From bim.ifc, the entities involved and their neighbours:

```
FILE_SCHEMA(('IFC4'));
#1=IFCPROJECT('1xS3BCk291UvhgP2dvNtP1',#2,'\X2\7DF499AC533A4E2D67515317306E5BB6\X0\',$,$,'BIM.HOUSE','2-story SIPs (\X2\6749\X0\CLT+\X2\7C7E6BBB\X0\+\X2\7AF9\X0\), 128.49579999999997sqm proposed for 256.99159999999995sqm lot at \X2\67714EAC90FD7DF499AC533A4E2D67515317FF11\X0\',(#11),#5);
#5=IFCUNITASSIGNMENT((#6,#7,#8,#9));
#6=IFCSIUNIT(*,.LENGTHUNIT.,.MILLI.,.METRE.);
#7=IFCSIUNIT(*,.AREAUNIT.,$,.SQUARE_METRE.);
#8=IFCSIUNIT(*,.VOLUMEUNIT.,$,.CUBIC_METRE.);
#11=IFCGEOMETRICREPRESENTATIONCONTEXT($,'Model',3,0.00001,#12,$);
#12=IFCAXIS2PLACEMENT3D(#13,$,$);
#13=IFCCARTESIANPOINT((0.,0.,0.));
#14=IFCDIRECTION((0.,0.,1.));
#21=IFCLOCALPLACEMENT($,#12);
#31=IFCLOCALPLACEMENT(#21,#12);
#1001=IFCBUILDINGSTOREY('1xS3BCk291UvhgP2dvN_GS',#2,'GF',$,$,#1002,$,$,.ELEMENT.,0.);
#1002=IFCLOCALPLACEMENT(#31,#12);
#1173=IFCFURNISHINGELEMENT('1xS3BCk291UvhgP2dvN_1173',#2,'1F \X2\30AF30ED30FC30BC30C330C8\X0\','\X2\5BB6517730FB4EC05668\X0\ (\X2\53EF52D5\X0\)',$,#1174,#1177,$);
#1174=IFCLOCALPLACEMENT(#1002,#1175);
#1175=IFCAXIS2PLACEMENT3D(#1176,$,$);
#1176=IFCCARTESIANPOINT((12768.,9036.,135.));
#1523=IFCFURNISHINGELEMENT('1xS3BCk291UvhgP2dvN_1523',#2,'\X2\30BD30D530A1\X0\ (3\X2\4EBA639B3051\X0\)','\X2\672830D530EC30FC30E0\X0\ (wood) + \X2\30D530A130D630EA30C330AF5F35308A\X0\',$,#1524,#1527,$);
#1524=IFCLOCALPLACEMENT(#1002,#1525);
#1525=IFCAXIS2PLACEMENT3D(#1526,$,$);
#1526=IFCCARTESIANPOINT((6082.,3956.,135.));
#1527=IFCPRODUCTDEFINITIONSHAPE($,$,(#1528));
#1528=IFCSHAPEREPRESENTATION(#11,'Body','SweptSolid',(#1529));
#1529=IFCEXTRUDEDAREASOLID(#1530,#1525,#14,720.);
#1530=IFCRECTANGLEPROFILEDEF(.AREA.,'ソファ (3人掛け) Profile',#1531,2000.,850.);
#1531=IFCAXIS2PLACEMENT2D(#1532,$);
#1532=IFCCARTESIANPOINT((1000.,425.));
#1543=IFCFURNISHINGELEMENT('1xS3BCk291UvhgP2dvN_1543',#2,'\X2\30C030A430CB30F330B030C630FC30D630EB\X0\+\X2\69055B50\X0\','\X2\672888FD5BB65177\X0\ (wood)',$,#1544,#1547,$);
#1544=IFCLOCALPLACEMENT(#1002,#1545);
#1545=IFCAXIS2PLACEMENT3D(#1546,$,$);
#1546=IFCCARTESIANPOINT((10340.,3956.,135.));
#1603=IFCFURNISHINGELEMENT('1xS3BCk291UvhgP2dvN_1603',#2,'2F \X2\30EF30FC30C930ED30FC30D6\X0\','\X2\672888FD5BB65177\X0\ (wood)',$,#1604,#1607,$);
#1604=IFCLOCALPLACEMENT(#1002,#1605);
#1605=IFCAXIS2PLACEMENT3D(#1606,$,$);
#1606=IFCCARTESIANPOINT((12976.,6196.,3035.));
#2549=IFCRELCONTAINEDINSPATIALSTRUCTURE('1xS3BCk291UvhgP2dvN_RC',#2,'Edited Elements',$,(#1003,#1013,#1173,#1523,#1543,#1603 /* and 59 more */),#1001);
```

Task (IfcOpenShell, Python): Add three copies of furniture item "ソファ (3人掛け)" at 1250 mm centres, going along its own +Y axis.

```python
import ifcopenshell
import ifcopenshell.api.geometry
import ifcopenshell.api.root
import ifcopenshell.util.element
import ifcopenshell.util.placement
import ifcopenshell.util.unit

model = ifcopenshell.open("bim.ifc")
unit_scale = ifcopenshell.util.unit.calculate_unit_scale(model)


def reuse_history(source, copy):
    """copy_class also copies each property set's owner history, people and application; keep the originals."""
    for rel in copy.IsDefinedBy:
        if rel.is_a("IfcRelDefinesByProperties") and (history := rel.RelatingPropertyDefinition.OwnerHistory):
            rel.RelatingPropertyDefinition.OwnerHistory = source.OwnerHistory
            ifcopenshell.util.element.remove_deep2(model, history)


source = model.by_id(1523)
base = ifcopenshell.util.placement.get_local_placement(source.ObjectPlacement)
step = base[:3, 1] * 1.25 / unit_scale

for i in range(1, 4):
    copy = ifcopenshell.api.root.copy_class(model, product=source)
    copy.Representation = ifcopenshell.util.element.copy_deep(
        model, source.Representation, exclude=["IfcGeometricRepresentationContext", "IfcRepresentationMap"]
    )
    reuse_history(source, copy)
    matrix = base.copy()
    matrix[:3, 3] += i * step
    print("added at", matrix[:3, 3].round(3) + 0.0)
    ifcopenshell.api.geometry.edit_object_placement(model, product=copy, matrix=matrix, is_si=False)

model.write("bim_updated.ifc")
```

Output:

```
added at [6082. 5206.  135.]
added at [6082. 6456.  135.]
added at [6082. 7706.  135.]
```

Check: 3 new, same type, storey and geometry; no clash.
